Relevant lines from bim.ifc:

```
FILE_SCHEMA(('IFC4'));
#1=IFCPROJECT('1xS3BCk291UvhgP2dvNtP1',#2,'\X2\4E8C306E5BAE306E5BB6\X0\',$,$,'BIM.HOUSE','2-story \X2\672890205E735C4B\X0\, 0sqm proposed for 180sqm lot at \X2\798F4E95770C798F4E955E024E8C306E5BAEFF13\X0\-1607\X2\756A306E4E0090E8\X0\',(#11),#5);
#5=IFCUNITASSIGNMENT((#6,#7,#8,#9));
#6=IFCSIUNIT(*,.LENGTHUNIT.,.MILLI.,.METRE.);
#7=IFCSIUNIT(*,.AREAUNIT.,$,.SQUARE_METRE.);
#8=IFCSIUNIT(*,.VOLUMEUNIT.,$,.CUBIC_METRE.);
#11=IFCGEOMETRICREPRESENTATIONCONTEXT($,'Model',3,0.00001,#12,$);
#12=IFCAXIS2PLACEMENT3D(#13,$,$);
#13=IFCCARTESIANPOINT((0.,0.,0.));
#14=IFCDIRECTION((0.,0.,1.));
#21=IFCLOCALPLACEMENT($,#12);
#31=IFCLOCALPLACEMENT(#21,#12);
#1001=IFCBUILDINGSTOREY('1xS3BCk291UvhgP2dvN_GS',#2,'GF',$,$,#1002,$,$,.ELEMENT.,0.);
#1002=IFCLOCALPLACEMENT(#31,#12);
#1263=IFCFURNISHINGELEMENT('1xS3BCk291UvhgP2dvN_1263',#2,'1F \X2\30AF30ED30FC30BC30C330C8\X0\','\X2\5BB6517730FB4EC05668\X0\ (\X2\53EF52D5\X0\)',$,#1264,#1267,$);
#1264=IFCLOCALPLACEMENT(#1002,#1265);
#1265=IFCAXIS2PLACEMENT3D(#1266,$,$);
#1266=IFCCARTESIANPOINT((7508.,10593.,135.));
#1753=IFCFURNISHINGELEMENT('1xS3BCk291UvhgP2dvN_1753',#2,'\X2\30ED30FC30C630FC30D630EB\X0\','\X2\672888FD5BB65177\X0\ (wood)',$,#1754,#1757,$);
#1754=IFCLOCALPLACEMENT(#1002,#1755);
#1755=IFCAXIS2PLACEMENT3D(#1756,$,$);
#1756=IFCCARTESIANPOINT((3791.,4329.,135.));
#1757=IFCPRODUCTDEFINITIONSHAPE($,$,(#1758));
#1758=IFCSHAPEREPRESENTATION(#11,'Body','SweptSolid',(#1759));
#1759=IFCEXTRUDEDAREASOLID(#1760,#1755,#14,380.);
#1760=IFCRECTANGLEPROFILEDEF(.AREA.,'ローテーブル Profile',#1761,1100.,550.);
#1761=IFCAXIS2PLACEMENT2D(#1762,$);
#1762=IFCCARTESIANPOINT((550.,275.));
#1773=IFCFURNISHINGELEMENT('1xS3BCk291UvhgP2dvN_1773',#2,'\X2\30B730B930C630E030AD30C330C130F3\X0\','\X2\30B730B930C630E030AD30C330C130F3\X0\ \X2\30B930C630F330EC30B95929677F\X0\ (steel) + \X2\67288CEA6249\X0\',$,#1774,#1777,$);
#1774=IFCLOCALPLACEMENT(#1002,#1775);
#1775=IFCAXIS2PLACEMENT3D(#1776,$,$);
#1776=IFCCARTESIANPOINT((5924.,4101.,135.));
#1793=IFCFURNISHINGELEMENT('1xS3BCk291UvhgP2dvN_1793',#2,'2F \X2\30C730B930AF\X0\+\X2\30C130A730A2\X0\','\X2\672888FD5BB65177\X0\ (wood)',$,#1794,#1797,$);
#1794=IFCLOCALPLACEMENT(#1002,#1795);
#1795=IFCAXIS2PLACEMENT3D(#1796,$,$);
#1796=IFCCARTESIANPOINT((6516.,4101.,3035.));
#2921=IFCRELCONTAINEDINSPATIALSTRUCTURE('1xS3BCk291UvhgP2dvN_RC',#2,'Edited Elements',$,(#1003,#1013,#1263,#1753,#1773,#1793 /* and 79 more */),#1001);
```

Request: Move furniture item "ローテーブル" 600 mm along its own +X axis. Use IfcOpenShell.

```python
import ifcopenshell
import ifcopenshell.api.geometry
import ifcopenshell.util.placement

model = ifcopenshell.open("bim.ifc")

item = model.by_id(1753)
matrix = ifcopenshell.util.placement.get_local_placement(item.ObjectPlacement)
matrix[:3, 3] += matrix[:3, 0] * 600.0
ifcopenshell.api.geometry.edit_object_placement(model, product=item, matrix=matrix, is_si=False)

print(ifcopenshell.util.placement.get_local_placement(item.ObjectPlacement).round(3) + 0.0)

model.write("bim_rev.ifc")
```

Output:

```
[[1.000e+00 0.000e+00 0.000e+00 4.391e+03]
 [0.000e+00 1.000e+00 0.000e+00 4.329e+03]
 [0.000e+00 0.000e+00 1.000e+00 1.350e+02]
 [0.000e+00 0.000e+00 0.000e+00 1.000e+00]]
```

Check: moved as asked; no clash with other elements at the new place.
